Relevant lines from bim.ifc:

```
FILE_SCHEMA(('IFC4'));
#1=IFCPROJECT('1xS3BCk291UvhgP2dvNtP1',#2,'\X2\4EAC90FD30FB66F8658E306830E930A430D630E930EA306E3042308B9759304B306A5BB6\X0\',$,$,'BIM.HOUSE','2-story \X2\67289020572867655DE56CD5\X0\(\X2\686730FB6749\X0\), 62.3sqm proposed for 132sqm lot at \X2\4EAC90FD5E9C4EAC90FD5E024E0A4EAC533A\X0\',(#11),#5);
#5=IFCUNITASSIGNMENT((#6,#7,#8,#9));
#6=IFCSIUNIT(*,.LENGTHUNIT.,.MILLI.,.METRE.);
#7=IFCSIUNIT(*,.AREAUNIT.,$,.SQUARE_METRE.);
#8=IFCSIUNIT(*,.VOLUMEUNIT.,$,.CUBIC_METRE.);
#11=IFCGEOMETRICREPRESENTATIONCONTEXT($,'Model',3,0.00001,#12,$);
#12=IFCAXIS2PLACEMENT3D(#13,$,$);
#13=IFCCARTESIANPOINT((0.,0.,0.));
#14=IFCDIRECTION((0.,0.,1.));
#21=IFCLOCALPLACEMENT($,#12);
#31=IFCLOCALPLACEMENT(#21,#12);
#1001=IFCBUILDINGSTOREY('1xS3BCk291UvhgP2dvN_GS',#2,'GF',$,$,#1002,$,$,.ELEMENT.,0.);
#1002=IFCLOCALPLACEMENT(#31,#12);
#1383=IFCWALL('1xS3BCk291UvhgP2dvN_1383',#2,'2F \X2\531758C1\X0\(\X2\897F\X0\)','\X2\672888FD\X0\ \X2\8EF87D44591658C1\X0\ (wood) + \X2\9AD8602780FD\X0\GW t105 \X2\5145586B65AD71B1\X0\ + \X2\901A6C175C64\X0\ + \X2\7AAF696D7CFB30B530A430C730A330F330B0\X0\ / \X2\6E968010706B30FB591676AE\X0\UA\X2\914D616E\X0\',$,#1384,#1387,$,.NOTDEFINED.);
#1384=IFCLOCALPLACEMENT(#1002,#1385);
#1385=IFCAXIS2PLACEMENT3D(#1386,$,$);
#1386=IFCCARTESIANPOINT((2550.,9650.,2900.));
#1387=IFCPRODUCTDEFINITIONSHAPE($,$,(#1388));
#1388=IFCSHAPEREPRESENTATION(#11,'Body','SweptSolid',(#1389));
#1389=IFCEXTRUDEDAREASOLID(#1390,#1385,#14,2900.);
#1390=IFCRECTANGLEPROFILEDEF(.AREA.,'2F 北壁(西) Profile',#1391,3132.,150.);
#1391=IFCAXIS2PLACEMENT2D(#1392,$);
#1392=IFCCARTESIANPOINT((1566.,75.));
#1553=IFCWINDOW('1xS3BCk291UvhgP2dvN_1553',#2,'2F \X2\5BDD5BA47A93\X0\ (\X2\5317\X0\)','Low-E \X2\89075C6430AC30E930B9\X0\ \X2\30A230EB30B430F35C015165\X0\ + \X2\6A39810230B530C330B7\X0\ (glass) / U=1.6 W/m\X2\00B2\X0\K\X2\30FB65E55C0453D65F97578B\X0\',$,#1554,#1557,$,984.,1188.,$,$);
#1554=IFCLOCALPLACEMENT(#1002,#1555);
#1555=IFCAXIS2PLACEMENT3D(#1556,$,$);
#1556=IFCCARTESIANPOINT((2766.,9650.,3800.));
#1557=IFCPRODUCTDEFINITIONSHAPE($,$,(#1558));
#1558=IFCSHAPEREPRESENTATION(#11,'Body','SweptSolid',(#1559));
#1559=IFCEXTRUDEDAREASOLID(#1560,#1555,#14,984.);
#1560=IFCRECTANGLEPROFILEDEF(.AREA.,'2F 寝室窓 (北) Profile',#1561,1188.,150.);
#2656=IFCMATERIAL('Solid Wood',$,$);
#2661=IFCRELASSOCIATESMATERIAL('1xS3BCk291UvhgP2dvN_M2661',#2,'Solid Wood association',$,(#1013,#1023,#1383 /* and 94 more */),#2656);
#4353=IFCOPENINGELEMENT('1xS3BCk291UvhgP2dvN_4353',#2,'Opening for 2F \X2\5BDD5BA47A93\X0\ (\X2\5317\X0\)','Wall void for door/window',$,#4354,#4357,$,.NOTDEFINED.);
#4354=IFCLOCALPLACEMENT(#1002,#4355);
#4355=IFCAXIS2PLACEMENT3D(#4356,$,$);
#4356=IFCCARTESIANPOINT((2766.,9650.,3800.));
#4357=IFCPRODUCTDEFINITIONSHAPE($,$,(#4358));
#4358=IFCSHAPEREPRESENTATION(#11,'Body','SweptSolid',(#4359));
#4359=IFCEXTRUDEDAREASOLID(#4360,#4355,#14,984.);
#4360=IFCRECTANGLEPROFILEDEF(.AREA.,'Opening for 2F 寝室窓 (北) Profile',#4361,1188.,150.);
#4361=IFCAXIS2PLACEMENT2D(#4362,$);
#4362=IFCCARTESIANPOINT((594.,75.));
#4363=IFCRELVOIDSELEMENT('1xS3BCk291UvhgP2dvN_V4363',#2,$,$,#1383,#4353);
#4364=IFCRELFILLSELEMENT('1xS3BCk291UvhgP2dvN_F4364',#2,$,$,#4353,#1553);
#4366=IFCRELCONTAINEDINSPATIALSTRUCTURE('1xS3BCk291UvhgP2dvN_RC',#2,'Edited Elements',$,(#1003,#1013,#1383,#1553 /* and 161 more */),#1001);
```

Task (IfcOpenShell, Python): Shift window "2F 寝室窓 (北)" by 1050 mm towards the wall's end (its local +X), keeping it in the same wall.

```python
import ifcopenshell
import ifcopenshell.api.geometry
import ifcopenshell.util.placement
import ifcopenshell.util.unit

model = ifcopenshell.open("bim.ifc")
unit_scale = ifcopenshell.util.unit.calculate_unit_scale(model)

window = model.by_guid("1xS3BCk291UvhgP2dvN_1553")
opening = window.FillsVoids[0].RelatingOpeningElement
wall = opening.VoidsElements[0].RelatingBuildingElement

wall_matrix = ifcopenshell.util.placement.get_local_placement(wall.ObjectPlacement)
shift = wall_matrix[:3, 0] * 1.05 / unit_scale
before = ifcopenshell.util.placement.get_local_placement(window.ObjectPlacement)[:3, 3].copy()

# The window is not placed relative to its opening, so move both.
for product in (opening, window):
    matrix = ifcopenshell.util.placement.get_local_placement(product.ObjectPlacement)
    matrix[:3, 3] += shift
    ifcopenshell.api.geometry.edit_object_placement(model, product=product, matrix=matrix, is_si=False)

after = ifcopenshell.util.placement.get_local_placement(window.ObjectPlacement)[:3, 3]
print("window moved by", (after - before).round(3) + 0.0)

model.write("bim_rev.ifc")
```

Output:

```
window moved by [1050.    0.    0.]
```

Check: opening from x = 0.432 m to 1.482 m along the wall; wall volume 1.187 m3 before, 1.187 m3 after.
